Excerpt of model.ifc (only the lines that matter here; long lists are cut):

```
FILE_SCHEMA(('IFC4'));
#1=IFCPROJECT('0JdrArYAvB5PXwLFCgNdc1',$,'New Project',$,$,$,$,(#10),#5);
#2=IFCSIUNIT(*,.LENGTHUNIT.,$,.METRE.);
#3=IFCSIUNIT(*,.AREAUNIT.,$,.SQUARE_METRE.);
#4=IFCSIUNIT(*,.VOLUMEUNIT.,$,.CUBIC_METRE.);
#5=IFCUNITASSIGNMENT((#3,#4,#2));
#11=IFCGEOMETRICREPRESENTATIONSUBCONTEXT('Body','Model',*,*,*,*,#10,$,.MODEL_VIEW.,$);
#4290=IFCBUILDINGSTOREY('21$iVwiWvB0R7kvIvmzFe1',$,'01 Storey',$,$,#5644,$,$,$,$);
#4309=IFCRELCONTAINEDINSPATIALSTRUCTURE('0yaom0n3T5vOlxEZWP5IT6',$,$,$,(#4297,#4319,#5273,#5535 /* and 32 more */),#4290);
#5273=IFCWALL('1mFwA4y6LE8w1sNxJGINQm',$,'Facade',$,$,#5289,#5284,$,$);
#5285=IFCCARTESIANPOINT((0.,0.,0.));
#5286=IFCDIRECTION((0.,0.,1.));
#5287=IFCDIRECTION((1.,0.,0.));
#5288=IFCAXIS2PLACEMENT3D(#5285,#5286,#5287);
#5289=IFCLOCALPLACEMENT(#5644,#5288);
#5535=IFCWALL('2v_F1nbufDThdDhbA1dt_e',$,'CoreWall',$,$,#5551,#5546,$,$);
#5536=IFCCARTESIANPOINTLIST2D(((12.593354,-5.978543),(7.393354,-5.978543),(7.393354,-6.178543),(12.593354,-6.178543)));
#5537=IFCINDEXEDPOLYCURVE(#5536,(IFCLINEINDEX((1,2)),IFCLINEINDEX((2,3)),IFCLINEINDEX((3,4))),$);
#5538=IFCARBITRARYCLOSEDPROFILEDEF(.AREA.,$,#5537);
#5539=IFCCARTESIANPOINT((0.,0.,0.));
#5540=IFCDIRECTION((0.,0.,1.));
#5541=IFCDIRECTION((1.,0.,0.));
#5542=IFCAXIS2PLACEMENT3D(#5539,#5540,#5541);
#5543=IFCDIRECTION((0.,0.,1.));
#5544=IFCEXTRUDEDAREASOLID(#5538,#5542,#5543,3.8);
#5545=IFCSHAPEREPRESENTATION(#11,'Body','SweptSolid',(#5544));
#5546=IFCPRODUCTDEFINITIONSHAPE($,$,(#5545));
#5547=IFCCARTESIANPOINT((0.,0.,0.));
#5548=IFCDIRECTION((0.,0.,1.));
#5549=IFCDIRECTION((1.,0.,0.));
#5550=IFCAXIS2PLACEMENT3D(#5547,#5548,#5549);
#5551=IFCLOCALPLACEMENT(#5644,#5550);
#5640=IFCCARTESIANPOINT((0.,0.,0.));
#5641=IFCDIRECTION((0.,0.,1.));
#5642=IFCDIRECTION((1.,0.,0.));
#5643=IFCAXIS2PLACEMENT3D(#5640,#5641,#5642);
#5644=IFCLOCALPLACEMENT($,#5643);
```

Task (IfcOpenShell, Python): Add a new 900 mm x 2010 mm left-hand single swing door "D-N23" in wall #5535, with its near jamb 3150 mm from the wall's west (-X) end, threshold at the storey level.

```python
import numpy as np
import ifcopenshell
import ifcopenshell.api.feature
import ifcopenshell.api.geometry
import ifcopenshell.api.root
import ifcopenshell.api.spatial
import ifcopenshell.geom
import ifcopenshell.util.element
import ifcopenshell.util.placement
import ifcopenshell.util.representation
import ifcopenshell.util.shape
import ifcopenshell.util.unit

model = ifcopenshell.open("model.ifc")
unit_scale = ifcopenshell.util.unit.calculate_unit_scale(model)
settings = ifcopenshell.geom.settings()


def volume(element):
    """Net volume in cubic metres, openings subtracted."""
    shape = ifcopenshell.geom.create_shape(settings, element)
    return ifcopenshell.util.shape.get_volume(shape.geometry)


wall = model.by_guid("2v_F1nbufDThdDhbA1dt_e")
storey = ifcopenshell.util.element.get_container(wall, ifc_class="IfcBuildingStorey")
context = ifcopenshell.util.representation.get_context(model, "Model", "Body", "MODEL_VIEW")
before = volume(wall)

width, height, from_end, sill = 0.9, 2.01, 3.15, 0.0  # metres

# The wall runs along its own X axis, and the end named is its -X end.
wall_shape = ifcopenshell.geom.create_shape(settings, wall)
x, y, z = ifcopenshell.util.shape.get_vertices(wall_shape.geometry).T
start = x.min() + from_end
face, thickness = float(y.min()), float(y.max() - y.min())
wall_matrix = ifcopenshell.util.placement.get_local_placement(wall.ObjectPlacement)
level = ifcopenshell.util.placement.get_local_placement(storey.ObjectPlacement)[2, 3]


def in_wall(x, y):
    """Placement at x, y metres in the wall's axes, at sill height."""
    matrix = wall_matrix.copy()
    matrix[:, 3] = wall_matrix @ np.array([x / unit_scale, y / unit_scale, 0.0, 1.0])
    matrix[2, 3] = level + sill / unit_scale
    return matrix


# Opening: a box that overshoots both wall faces by 50 mm.
opening = ifcopenshell.api.root.create_entity(model, ifc_class="IfcOpeningElement", predefined_type="OPENING")
box = ifcopenshell.api.geometry.add_wall_representation(
    model, context=context, length=width, height=height, thickness=thickness + 0.1
)
ifcopenshell.api.geometry.assign_representation(model, product=opening, representation=box)
ifcopenshell.api.geometry.edit_object_placement(model, product=opening, matrix=in_wall(start, face - 0.05), is_si=False)
ifcopenshell.api.feature.add_feature(model, feature=opening, element=wall)

door = ifcopenshell.api.root.create_entity(model, ifc_class="IfcDoor", name="D-N23", predefined_type="DOOR")
door.OverallWidth, door.OverallHeight = width / unit_scale, height / unit_scale
door.OperationType = "SINGLE_SWING_LEFT"
body = ifcopenshell.api.geometry.add_door_representation(
    model,
    context=context,
    overall_width=door.OverallWidth,
    overall_height=door.OverallHeight,
    operation_type="SINGLE_SWING_LEFT",
    lining_properties={"LiningDepth": thickness / unit_scale, "ThresholdDepth": thickness / unit_scale},
)
ifcopenshell.api.geometry.assign_representation(model, product=door, representation=body)
ifcopenshell.api.spatial.assign_container(model, products=[door], relating_structure=storey)
ifcopenshell.api.feature.add_filling(model, opening=opening, element=door)

# The lining spans the wall, so the door starts at the wall face.
ifcopenshell.api.geometry.edit_object_placement(model, product=door, matrix=in_wall(start, face), is_si=False)

after = volume(wall)

print(f"wall volume {before:.3f} -> {after:.3f} m3")

model.write("model_updated.ifc")
```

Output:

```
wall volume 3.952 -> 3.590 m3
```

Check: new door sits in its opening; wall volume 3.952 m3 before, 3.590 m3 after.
